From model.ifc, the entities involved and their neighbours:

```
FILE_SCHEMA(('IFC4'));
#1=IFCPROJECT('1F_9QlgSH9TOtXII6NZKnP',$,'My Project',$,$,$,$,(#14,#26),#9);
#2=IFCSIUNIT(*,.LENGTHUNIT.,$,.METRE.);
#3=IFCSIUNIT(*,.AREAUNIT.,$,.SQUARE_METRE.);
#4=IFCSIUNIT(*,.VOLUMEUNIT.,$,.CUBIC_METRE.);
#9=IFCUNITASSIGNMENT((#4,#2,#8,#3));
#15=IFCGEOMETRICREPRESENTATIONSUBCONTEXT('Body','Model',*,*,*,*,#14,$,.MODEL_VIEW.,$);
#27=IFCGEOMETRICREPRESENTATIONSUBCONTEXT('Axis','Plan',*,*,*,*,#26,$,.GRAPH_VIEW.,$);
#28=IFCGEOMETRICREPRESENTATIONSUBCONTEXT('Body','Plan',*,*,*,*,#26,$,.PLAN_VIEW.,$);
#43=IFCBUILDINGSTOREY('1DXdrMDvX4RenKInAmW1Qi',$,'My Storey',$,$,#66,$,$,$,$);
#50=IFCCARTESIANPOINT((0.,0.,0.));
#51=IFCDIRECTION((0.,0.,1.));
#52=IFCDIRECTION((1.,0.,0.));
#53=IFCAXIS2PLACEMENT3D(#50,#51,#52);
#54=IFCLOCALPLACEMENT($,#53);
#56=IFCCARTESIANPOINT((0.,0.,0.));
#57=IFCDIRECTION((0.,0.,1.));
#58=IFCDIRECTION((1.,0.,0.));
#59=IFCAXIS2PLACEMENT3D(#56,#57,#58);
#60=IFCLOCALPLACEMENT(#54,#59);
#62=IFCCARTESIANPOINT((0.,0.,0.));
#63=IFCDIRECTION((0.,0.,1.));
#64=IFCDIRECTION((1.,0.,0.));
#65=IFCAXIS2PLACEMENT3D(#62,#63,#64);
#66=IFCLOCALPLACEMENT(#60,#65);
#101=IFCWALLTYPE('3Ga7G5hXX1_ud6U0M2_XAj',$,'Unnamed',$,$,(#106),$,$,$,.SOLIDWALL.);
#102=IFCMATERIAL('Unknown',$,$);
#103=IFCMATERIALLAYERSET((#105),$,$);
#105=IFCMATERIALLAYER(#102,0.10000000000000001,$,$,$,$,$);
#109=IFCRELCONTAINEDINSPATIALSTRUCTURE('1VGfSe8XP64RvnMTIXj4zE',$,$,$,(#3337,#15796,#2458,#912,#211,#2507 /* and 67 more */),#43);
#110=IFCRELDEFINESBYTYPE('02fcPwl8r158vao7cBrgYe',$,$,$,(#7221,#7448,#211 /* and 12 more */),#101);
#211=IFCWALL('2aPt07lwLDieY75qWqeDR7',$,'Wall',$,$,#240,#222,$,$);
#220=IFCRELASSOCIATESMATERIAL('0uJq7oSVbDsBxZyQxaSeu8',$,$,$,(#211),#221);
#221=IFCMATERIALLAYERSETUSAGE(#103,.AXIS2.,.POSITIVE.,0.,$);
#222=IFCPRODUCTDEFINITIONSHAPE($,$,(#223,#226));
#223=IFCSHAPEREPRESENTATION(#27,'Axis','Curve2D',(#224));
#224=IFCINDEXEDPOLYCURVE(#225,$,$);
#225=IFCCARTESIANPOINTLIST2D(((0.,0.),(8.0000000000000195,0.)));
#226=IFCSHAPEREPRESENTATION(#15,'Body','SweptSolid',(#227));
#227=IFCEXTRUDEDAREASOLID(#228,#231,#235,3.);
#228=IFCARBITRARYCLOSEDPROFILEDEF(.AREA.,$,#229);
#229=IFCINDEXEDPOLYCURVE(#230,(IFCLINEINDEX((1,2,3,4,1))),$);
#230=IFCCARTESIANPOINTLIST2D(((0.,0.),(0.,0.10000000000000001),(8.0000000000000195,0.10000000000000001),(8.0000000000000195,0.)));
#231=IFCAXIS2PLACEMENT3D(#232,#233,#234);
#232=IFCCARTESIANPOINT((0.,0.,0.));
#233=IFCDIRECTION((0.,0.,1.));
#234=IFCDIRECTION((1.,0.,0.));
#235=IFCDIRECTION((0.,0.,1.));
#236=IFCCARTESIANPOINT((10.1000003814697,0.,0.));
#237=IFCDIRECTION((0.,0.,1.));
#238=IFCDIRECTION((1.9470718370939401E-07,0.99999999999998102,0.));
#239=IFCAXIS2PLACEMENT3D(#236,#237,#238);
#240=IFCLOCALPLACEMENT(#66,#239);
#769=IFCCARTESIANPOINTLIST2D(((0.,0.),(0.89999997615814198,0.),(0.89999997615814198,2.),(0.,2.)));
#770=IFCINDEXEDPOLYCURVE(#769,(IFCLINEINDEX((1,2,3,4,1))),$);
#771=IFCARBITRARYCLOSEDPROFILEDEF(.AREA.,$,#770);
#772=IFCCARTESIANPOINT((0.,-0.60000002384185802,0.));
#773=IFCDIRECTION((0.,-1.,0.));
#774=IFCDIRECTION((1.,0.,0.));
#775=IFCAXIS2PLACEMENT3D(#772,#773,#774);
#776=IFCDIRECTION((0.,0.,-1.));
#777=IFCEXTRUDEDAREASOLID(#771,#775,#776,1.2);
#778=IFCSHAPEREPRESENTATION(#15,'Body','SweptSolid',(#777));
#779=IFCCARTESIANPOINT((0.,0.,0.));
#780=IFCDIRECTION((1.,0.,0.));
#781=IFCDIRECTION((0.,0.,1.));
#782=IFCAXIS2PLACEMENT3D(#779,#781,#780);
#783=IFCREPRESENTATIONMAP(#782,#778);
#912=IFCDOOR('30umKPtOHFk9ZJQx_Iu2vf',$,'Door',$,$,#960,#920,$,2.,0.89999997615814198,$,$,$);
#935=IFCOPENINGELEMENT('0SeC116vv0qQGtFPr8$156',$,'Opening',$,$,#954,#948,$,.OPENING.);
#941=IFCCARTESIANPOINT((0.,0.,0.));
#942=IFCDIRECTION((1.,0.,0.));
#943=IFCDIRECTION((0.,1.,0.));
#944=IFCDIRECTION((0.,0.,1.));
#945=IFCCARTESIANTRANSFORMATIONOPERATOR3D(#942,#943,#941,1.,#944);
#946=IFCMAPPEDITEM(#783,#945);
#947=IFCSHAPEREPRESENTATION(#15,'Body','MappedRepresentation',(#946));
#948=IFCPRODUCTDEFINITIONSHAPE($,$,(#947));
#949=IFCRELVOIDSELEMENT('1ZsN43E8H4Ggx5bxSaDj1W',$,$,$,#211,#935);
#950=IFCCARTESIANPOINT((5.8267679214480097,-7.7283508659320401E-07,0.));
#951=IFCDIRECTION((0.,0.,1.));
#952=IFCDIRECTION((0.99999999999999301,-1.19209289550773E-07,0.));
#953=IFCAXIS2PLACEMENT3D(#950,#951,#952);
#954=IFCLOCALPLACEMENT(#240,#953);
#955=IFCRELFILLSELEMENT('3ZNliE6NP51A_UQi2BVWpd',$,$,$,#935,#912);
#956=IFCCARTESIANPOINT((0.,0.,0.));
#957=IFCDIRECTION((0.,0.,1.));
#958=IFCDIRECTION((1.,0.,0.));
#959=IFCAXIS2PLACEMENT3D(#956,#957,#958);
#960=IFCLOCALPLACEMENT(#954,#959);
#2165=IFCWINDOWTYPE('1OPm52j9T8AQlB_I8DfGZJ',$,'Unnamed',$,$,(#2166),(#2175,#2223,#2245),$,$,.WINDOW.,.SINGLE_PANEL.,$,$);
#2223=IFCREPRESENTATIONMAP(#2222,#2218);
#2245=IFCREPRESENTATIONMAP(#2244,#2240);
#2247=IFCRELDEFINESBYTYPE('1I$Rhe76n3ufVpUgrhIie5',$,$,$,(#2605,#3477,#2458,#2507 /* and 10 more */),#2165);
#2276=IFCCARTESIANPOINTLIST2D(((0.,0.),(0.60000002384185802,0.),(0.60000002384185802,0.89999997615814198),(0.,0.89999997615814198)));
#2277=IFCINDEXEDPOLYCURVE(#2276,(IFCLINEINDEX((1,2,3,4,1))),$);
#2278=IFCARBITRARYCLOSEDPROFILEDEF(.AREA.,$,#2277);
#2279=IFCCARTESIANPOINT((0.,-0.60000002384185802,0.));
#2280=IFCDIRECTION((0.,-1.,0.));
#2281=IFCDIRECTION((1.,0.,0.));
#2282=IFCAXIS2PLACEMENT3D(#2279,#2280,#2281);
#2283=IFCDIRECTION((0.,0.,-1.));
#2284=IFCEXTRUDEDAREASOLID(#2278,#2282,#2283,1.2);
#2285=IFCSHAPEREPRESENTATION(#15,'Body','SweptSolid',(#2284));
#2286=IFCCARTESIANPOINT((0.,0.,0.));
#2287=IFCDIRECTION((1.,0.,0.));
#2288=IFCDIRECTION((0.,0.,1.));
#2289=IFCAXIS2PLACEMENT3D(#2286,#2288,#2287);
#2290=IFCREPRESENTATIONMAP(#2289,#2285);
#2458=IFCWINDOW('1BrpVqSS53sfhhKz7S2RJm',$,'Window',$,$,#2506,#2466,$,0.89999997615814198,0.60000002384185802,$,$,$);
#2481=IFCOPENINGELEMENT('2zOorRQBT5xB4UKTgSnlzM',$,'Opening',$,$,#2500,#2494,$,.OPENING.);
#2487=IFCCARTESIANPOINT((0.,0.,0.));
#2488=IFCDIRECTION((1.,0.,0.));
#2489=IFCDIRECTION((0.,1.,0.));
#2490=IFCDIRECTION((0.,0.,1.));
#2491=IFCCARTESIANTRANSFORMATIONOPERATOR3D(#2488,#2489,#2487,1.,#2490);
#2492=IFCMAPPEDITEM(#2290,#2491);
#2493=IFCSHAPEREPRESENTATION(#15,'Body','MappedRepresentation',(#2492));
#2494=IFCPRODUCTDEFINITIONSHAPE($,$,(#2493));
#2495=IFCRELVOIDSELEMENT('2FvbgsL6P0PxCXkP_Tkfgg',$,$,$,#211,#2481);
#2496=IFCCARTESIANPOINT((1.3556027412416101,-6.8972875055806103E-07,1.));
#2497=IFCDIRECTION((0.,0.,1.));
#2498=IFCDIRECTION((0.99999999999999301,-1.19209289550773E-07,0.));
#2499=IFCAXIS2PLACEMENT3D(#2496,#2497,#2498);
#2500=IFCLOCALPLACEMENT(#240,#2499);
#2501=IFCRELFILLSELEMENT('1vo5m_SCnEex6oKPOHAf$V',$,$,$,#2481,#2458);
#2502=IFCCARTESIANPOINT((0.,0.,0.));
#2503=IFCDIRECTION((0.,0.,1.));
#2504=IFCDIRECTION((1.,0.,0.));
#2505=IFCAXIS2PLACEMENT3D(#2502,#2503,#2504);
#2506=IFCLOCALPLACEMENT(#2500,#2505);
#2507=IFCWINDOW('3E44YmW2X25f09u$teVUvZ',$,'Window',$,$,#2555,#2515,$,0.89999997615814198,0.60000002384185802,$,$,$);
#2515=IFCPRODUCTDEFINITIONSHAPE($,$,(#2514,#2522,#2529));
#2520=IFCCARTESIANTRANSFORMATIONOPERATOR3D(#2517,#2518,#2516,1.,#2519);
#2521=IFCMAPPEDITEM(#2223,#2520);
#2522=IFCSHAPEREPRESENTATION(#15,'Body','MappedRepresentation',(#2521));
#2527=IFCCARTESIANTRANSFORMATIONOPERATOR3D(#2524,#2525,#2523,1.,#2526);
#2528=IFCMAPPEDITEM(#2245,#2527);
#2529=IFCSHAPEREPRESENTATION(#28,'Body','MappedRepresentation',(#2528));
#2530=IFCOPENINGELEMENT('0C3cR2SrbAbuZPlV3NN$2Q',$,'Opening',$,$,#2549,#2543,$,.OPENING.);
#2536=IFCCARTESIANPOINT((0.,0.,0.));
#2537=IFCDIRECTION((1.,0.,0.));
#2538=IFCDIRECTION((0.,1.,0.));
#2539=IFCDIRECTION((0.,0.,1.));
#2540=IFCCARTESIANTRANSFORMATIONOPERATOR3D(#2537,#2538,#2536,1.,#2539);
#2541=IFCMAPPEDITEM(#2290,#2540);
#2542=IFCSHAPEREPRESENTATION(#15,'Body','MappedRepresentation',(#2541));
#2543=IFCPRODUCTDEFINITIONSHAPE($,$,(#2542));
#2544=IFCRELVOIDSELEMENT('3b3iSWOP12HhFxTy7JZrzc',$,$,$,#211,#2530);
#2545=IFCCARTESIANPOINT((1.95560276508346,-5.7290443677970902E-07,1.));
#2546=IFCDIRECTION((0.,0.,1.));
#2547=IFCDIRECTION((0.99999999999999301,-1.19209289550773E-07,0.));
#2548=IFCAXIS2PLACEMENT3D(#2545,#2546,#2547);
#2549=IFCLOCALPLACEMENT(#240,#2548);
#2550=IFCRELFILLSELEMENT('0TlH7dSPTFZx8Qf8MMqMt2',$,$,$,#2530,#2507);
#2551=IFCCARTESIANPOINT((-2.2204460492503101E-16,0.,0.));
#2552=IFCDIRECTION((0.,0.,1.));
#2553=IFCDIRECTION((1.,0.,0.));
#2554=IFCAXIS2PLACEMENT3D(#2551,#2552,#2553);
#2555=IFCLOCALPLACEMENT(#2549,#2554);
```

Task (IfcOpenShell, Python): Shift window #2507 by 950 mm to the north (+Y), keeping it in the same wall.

```python
import ifcopenshell
import ifcopenshell.api.geometry
import ifcopenshell.util.placement

model = ifcopenshell.open("model.ifc")

window = model.by_guid("3E44YmW2X25f09u$teVUvZ")
opening = window.FillsVoids[0].RelatingOpeningElement
wall = opening.VoidsElements[0].RelatingBuildingElement

wall_matrix = ifcopenshell.util.placement.get_local_placement(wall.ObjectPlacement)
shift = wall_matrix[:3, 0] * 0.95
before = ifcopenshell.util.placement.get_local_placement(window.ObjectPlacement)[:3, 3].copy()

# The window is placed relative to its opening, so it follows when the opening moves.
matrix = ifcopenshell.util.placement.get_local_placement(opening.ObjectPlacement)
matrix[:3, 3] += shift
ifcopenshell.api.geometry.edit_object_placement(
    model, product=opening, matrix=matrix, is_si=False, should_transform_children=True
)

after = ifcopenshell.util.placement.get_local_placement(window.ObjectPlacement)[:3, 3]
print("window moved by", (after - before).round(3) + 0.0)

model.write("model_updated.ifc")
```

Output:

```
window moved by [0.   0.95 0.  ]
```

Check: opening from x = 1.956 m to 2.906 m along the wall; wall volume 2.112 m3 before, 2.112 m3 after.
